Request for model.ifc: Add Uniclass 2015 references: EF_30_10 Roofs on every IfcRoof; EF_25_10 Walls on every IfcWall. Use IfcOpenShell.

First a look at what the model holds.

```python
import ifcopenshell

model = ifcopenshell.open("model.ifc")
print(model.schema)
print("classifications:", [c.Name for c in model.by_type("IfcClassification")])
for ifc_class in ("IfcDoor", "IfcRoof", "IfcStair", "IfcWall", "IfcWindow"):
    print(ifc_class, len(model.by_type(ifc_class)))
```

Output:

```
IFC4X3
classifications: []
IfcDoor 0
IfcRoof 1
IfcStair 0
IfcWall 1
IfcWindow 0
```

```python
import ifcopenshell
import ifcopenshell.api.classification

model = ifcopenshell.open("model.ifc")

system = ifcopenshell.api.classification.add_classification(model, classification="Uniclass 2015")

codes = {
    "IfcRoof": ("EF_30_10", "Roofs"),
    "IfcWall": ("EF_25_10", "Walls"),
}
for ifc_class, (code, name) in codes.items():
    products = model.by_type(ifc_class)
    ifcopenshell.api.classification.add_reference(
        model, products=products, classification=system, identification=code, name=name
    )
    print(code, len(products))

model.write("model_v2.ifc")
```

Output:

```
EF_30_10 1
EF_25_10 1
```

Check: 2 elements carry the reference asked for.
